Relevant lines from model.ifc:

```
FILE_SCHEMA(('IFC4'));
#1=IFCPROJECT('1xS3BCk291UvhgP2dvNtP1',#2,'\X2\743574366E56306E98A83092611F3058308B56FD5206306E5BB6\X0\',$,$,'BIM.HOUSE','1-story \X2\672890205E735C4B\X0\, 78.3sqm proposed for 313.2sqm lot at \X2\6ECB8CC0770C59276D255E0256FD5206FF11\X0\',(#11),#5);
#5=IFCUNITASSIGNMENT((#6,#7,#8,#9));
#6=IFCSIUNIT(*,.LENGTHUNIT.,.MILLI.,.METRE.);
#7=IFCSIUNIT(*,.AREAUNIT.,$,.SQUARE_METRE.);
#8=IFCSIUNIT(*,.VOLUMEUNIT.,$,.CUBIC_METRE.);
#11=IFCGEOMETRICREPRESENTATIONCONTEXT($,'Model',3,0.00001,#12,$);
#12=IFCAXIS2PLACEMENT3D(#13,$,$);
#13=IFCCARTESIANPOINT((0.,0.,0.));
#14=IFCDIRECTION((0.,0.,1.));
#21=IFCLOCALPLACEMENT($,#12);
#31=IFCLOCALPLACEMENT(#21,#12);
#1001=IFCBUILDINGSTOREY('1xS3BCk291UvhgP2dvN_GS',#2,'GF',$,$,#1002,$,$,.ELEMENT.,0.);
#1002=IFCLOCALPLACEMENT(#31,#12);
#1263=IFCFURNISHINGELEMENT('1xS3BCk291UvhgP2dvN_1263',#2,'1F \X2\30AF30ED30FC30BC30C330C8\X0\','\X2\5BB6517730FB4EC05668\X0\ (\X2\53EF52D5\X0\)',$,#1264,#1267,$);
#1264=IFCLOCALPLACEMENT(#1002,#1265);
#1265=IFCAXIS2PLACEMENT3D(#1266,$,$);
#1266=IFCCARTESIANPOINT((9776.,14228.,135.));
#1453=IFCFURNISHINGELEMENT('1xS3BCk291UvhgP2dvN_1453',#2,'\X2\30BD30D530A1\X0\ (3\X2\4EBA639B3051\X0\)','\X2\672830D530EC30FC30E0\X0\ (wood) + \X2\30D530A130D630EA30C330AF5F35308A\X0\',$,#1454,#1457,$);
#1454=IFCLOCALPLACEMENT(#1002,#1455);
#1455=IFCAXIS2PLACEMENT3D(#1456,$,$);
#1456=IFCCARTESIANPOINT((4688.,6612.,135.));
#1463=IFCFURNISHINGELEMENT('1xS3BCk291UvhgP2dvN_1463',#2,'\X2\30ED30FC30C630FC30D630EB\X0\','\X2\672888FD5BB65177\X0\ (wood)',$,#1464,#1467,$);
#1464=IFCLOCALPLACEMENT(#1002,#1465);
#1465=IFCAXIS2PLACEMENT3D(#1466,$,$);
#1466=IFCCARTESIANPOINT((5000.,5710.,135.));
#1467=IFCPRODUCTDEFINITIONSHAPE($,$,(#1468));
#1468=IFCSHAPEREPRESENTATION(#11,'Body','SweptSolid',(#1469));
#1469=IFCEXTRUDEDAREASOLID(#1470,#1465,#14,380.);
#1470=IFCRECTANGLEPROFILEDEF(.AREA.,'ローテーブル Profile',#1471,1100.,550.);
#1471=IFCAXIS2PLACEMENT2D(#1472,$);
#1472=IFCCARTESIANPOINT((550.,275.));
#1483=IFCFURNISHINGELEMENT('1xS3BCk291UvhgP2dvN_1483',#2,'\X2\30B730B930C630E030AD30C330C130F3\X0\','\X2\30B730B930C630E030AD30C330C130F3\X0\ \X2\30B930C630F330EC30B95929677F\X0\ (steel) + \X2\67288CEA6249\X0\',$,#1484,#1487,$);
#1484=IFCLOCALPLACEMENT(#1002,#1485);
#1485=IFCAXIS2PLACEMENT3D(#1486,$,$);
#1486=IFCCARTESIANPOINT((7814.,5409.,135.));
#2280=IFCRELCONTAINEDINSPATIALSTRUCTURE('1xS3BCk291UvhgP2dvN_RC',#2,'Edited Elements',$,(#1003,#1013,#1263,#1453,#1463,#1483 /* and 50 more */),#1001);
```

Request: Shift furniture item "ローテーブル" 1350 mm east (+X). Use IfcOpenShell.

```python
import ifcopenshell
import ifcopenshell.api.geometry
import ifcopenshell.util.placement
import ifcopenshell.util.unit

model = ifcopenshell.open("model.ifc")
unit_scale = ifcopenshell.util.unit.calculate_unit_scale(model)

item = model.by_guid("1xS3BCk291UvhgP2dvN_1463")
matrix = ifcopenshell.util.placement.get_local_placement(item.ObjectPlacement)
matrix[0, 3] += 1.35 / unit_scale
ifcopenshell.api.geometry.edit_object_placement(model, product=item, matrix=matrix, is_si=False)

print(ifcopenshell.util.placement.get_local_placement(item.ObjectPlacement).round(3) + 0.0)

model.write("model_rev.ifc")
```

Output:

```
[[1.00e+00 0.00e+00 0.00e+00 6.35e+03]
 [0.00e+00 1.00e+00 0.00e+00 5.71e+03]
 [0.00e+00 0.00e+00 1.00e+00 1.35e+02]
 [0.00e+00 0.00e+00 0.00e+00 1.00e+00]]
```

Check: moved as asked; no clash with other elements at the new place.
